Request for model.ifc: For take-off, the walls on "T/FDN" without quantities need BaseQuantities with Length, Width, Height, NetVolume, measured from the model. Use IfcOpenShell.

First a look at what the model holds.

```python
import ifcopenshell
import ifcopenshell.util.element
import ifcopenshell.util.unit

model = ifcopenshell.open("model.ifc")
print(model.schema)
for unit_type in ("LENGTHUNIT", "AREAUNIT", "VOLUMEUNIT"):
    print(unit_type, ifcopenshell.util.unit.calculate_unit_scale(model, unit_type))
storey = next(s for s in model.by_type("IfcBuildingStorey") if s.Name == "T/FDN")
walls = [e for e in ifcopenshell.util.element.get_decomposition(storey) if e.is_a("IfcWall")]
for e in sorted(walls, key=lambda e: e.id()):
    print(e.id(), e.is_a(), e.Name, list(ifcopenshell.util.element.get_psets(e, qtos_only=True)), sep=" | ")
```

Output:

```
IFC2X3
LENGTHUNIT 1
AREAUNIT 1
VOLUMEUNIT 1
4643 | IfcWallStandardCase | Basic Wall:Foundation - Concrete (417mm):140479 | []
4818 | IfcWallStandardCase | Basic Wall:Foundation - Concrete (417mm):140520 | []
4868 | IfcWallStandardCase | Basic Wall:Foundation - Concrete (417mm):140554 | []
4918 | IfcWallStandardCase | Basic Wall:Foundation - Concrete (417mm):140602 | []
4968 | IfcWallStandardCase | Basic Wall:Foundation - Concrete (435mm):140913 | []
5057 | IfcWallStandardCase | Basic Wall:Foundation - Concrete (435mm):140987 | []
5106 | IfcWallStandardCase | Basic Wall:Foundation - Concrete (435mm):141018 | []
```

```python
import ifcopenshell
import ifcopenshell.api.pset
import ifcopenshell.geom
import ifcopenshell.util.element
import ifcopenshell.util.shape
import ifcopenshell.util.unit

model = ifcopenshell.open("model.ifc")
unit_scale = ifcopenshell.util.unit.calculate_unit_scale(model)
volume_scale = ifcopenshell.util.unit.calculate_unit_scale(model, "VOLUMEUNIT")
settings = ifcopenshell.geom.settings()

storey = next(s for s in model.by_type("IfcBuildingStorey") if s.Name == "T/FDN")
walls = [e for e in ifcopenshell.util.element.get_decomposition(storey) if e.is_a("IfcWall")]

for e in sorted(walls, key=lambda e: e.id()):
    if ifcopenshell.util.element.get_psets(e, qtos_only=True, should_inherit=False):
        continue
    # Geometry comes back in metres, in the element's own axes.
    shape = ifcopenshell.geom.create_shape(settings, e)
    values = {
        "Length": ifcopenshell.util.shape.get_x(shape.geometry) / unit_scale,
        "Width": ifcopenshell.util.shape.get_y(shape.geometry) / unit_scale,
        "Height": ifcopenshell.util.shape.get_z(shape.geometry) / unit_scale,
        "NetVolume": ifcopenshell.util.shape.get_volume(shape.geometry) / volume_scale,
    }
    qto = ifcopenshell.api.pset.add_qto(model, product=e, name="BaseQuantities")
    ifcopenshell.api.pset.edit_qto(model, qto=qto, properties=values)
    print(e.id(), {k: round(v, 3) for k, v in values.items()})

model.write("model_v2.ifc")
```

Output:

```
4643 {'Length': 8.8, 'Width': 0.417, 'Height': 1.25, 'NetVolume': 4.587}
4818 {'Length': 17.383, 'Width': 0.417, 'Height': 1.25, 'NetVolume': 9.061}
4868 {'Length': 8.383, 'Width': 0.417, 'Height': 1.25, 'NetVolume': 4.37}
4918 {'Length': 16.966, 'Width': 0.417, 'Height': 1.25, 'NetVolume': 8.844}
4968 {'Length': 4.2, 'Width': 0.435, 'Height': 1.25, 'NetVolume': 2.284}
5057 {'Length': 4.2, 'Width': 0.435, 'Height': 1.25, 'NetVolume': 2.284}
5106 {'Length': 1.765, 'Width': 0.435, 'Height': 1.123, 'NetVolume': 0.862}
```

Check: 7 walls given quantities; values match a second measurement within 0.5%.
